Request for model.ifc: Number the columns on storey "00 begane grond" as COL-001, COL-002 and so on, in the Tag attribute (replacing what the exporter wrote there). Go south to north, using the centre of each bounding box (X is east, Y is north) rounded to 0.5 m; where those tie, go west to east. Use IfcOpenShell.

First a look at what the model holds.

```python
import ifcopenshell
import ifcopenshell.util.element
import ifcopenshell.util.placement

model = ifcopenshell.open("model.ifc")
print(model.schema)
storey = next(s for s in model.by_type("IfcBuildingStorey") if s.Name == "00 begane grond")
columns = [e for e in ifcopenshell.util.element.get_decomposition(storey) if e.is_a("IfcColumn")]
for e in sorted(columns, key=lambda e: e.id()):
    origin = ifcopenshell.util.placement.get_local_placement(e.ObjectPlacement)[:3, 3]
    print(e.id(), e.Tag, e.Name, origin.round(2) + 0.0, sep=" | ")
```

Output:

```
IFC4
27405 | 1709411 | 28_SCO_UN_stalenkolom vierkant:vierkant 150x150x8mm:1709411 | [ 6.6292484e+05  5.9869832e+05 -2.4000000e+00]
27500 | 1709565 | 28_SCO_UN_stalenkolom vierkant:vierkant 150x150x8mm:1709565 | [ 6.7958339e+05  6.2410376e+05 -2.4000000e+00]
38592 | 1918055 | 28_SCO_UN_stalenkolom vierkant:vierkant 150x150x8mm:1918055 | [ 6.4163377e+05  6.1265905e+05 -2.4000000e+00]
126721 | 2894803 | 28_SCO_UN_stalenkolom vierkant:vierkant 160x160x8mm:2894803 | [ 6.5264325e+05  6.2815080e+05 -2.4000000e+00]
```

```python
import ifcopenshell
import ifcopenshell.geom
import ifcopenshell.util.element
import ifcopenshell.util.shape

model = ifcopenshell.open("model.ifc")
settings = ifcopenshell.geom.settings()
settings.set("use-world-coords", True)


def centre(element):
    shape = ifcopenshell.geom.create_shape(settings, element)
    return ifcopenshell.util.shape.get_bbox_centroid(shape.geometry)


storey = next(s for s in model.by_type("IfcBuildingStorey") if s.Name == "00 begane grond")
columns = [e for e in ifcopenshell.util.element.get_decomposition(storey) if e.is_a("IfcColumn")]

# Insertion points can sit at a corner or the storey origin, so sort by the geometry (in metres).
centres = {e: centre(e) for e in columns}
columns.sort(key=lambda e: (round(centres[e][1] / 0.5), centres[e][0]))

for i, e in enumerate(columns, start=1):
    number = f"COL-0{i:02d}"
    e.Tag = number
    print(e.id(), number)

model.write("model_v2.ifc")
```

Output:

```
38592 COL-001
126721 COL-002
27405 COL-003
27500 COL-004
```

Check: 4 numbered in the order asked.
